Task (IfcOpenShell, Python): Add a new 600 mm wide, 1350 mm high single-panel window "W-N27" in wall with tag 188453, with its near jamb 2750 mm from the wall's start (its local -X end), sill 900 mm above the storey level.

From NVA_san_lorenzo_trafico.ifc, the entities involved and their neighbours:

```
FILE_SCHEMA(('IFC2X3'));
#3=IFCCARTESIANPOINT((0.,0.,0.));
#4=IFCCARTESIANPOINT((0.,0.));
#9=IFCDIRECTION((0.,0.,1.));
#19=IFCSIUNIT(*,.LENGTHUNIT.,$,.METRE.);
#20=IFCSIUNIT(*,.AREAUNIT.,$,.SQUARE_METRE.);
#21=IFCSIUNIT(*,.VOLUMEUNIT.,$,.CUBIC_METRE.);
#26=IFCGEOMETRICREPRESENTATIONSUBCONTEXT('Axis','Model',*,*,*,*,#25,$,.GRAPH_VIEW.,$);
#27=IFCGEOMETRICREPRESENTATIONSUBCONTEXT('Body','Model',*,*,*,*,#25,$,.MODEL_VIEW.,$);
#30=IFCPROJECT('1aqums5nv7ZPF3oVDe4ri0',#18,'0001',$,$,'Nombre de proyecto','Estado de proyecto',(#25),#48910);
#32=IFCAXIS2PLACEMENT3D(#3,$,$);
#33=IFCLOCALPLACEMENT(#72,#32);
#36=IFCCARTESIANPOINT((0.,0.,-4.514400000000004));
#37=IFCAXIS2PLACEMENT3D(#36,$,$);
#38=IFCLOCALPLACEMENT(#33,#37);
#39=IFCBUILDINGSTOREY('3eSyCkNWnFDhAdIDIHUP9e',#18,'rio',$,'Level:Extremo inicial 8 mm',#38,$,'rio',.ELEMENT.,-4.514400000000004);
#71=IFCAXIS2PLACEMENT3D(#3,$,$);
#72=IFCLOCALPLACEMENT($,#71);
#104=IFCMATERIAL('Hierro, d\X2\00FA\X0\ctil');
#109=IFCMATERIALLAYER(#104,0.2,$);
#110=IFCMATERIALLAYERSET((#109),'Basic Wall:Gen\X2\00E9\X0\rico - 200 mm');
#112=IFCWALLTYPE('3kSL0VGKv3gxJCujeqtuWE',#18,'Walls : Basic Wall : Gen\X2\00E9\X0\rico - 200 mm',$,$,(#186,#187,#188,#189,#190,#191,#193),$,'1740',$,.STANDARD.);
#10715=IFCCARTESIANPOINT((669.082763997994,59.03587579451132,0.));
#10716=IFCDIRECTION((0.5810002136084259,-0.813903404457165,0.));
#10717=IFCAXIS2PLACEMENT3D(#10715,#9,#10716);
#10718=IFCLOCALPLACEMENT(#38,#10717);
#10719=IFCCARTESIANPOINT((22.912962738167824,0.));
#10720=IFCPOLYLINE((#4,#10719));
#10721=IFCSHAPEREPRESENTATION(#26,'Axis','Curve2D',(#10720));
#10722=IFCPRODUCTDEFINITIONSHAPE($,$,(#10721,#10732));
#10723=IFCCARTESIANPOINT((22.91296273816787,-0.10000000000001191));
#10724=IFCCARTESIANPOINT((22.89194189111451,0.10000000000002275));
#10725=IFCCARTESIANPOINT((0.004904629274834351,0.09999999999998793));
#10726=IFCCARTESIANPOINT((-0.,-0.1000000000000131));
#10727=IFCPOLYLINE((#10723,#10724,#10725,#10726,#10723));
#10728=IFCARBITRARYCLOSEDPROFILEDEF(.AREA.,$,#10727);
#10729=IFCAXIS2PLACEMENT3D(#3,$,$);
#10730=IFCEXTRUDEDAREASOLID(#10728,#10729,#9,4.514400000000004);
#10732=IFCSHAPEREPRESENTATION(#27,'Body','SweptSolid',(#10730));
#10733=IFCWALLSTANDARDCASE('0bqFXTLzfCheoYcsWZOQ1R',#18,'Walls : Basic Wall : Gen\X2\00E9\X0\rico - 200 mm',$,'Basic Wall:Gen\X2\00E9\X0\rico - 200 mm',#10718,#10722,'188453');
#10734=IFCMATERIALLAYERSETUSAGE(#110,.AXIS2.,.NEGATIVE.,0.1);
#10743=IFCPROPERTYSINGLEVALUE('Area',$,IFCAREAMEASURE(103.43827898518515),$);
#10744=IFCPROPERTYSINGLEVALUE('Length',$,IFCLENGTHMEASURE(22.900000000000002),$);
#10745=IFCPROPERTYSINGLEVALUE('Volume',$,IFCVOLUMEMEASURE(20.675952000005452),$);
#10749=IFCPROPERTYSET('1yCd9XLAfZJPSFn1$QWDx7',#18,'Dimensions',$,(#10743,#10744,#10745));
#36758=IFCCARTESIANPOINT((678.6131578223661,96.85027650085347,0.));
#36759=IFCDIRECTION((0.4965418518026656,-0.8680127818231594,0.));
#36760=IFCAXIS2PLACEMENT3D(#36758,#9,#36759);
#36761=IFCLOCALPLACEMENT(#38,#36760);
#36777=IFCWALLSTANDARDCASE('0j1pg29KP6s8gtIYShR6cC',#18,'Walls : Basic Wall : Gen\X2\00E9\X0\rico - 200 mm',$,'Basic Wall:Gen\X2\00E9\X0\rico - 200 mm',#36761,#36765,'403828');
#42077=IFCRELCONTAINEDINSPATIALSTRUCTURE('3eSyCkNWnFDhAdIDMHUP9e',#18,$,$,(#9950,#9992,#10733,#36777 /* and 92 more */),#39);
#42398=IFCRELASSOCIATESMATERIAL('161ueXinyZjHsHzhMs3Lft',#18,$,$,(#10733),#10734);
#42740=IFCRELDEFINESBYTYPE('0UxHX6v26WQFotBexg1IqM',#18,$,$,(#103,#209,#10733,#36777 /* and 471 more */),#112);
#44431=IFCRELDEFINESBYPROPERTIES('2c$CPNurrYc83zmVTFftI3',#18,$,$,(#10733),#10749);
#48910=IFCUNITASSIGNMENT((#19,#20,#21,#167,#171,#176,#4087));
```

```python
import numpy as np
import ifcopenshell
import ifcopenshell.api.feature
import ifcopenshell.api.geometry
import ifcopenshell.api.pset
import ifcopenshell.api.root
import ifcopenshell.api.spatial
import ifcopenshell.api.type
import ifcopenshell.geom
import ifcopenshell.util.element
import ifcopenshell.util.placement
import ifcopenshell.util.representation
import ifcopenshell.util.shape
import ifcopenshell.util.unit

model = ifcopenshell.open("NVA_san_lorenzo_trafico.ifc")
unit_scale = ifcopenshell.util.unit.calculate_unit_scale(model)
area_scale = ifcopenshell.util.unit.calculate_unit_scale(model, "AREAUNIT")
volume_scale = ifcopenshell.util.unit.calculate_unit_scale(model, "VOLUMEUNIT")
settings = ifcopenshell.geom.settings()


def volume(element):
    """Net volume in cubic metres, openings subtracted."""
    shape = ifcopenshell.geom.create_shape(settings, element)
    return ifcopenshell.util.shape.get_volume(shape.geometry)


wall = model.by_guid("0bqFXTLzfCheoYcsWZOQ1R")
storey = ifcopenshell.util.element.get_container(wall, ifc_class="IfcBuildingStorey")
context = ifcopenshell.util.representation.get_context(model, "Model", "Body", "MODEL_VIEW")
before = volume(wall)

width, height, from_end, sill = 0.6, 1.35, 2.75, 0.9  # metres

# The wall runs along its own X axis, and the end named is its -X end.
wall_shape = ifcopenshell.geom.create_shape(settings, wall)
x, y, z = ifcopenshell.util.shape.get_vertices(wall_shape.geometry).T
start = x.min() + from_end
face, thickness = float(y.min()), float(y.max() - y.min())
wall_matrix = ifcopenshell.util.placement.get_local_placement(wall.ObjectPlacement)
level = ifcopenshell.util.placement.get_local_placement(storey.ObjectPlacement)[2, 3]


def in_wall(x, y):
    """Placement at x, y metres in the wall's axes, at sill height."""
    matrix = wall_matrix.copy()
    matrix[:, 3] = wall_matrix @ np.array([x / unit_scale, y / unit_scale, 0.0, 1.0])
    matrix[2, 3] = level + sill / unit_scale
    return matrix


# Opening: a box that overshoots both wall faces by 50 mm.
opening = ifcopenshell.api.root.create_entity(model, ifc_class="IfcOpeningElement")
box = ifcopenshell.api.geometry.add_wall_representation(
    model, context=context, length=width, height=height, thickness=thickness + 0.1
)
ifcopenshell.api.geometry.assign_representation(model, product=opening, representation=box)
ifcopenshell.api.geometry.edit_object_placement(model, product=opening, matrix=in_wall(start, face - 0.05), is_si=False)
ifcopenshell.api.feature.add_feature(model, feature=opening, element=wall)

window = ifcopenshell.api.root.create_entity(model, ifc_class="IfcWindow", name="W-N27")
window.OverallWidth, window.OverallHeight = width / unit_scale, height / unit_scale
body = ifcopenshell.api.geometry.add_window_representation(
    model,
    context=context,
    overall_width=window.OverallWidth,
    overall_height=window.OverallHeight,
    partition_type="SINGLE_PANEL",
)
ifcopenshell.api.geometry.assign_representation(model, product=window, representation=body)
ifcopenshell.api.spatial.assign_container(model, products=[window], relating_structure=storey)
fills = ifcopenshell.api.feature.add_filling(model, opening=opening, element=window)
fills.OwnerHistory = window.OwnerHistory  # required in IFC2X3

# IFC2X3 keeps the operation on the window style.
style = ifcopenshell.api.root.create_entity(model, ifc_class="IfcWindowStyle", name="W-N27")
style.OperationType, style.ConstructionType = "SINGLE_PANEL", "NOTDEFINED"
style.ParameterTakesPrecedence = style.Sizeable = False
ifcopenshell.api.type.assign_type(model, related_objects=[window], relating_type=style)

# Centre the window in the wall's thickness.
ifcopenshell.api.geometry.edit_object_placement(model, product=window, matrix=in_wall(start, face), is_si=False)
window_shape = ifcopenshell.geom.create_shape(settings, window)
depth = ifcopenshell.util.shape.get_vertices(window_shape.geometry)[:, 1]
offset = face + thickness / 2 - (depth.min() + depth.max()) / 2
ifcopenshell.api.geometry.edit_object_placement(model, product=window, matrix=in_wall(start, offset), is_si=False)

after = volume(wall)

# Update the wall's stored quantities.
pset = model.by_id(ifcopenshell.util.element.get_pset(wall, "Dimensions", should_inherit=False)["id"])
ifcopenshell.api.pset.edit_pset(model, pset=pset, properties={
    "Area": model.create_entity("IfcAreaMeasure", after / thickness / area_scale),
    "Volume": model.create_entity("IfcVolumeMeasure", after / volume_scale),
})

print(f"wall volume {before:.3f} -> {after:.3f} m3")

model.write("NVA_san_lorenzo_trafico_edited.ifc")
```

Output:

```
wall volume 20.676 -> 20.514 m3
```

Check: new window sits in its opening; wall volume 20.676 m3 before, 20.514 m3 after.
